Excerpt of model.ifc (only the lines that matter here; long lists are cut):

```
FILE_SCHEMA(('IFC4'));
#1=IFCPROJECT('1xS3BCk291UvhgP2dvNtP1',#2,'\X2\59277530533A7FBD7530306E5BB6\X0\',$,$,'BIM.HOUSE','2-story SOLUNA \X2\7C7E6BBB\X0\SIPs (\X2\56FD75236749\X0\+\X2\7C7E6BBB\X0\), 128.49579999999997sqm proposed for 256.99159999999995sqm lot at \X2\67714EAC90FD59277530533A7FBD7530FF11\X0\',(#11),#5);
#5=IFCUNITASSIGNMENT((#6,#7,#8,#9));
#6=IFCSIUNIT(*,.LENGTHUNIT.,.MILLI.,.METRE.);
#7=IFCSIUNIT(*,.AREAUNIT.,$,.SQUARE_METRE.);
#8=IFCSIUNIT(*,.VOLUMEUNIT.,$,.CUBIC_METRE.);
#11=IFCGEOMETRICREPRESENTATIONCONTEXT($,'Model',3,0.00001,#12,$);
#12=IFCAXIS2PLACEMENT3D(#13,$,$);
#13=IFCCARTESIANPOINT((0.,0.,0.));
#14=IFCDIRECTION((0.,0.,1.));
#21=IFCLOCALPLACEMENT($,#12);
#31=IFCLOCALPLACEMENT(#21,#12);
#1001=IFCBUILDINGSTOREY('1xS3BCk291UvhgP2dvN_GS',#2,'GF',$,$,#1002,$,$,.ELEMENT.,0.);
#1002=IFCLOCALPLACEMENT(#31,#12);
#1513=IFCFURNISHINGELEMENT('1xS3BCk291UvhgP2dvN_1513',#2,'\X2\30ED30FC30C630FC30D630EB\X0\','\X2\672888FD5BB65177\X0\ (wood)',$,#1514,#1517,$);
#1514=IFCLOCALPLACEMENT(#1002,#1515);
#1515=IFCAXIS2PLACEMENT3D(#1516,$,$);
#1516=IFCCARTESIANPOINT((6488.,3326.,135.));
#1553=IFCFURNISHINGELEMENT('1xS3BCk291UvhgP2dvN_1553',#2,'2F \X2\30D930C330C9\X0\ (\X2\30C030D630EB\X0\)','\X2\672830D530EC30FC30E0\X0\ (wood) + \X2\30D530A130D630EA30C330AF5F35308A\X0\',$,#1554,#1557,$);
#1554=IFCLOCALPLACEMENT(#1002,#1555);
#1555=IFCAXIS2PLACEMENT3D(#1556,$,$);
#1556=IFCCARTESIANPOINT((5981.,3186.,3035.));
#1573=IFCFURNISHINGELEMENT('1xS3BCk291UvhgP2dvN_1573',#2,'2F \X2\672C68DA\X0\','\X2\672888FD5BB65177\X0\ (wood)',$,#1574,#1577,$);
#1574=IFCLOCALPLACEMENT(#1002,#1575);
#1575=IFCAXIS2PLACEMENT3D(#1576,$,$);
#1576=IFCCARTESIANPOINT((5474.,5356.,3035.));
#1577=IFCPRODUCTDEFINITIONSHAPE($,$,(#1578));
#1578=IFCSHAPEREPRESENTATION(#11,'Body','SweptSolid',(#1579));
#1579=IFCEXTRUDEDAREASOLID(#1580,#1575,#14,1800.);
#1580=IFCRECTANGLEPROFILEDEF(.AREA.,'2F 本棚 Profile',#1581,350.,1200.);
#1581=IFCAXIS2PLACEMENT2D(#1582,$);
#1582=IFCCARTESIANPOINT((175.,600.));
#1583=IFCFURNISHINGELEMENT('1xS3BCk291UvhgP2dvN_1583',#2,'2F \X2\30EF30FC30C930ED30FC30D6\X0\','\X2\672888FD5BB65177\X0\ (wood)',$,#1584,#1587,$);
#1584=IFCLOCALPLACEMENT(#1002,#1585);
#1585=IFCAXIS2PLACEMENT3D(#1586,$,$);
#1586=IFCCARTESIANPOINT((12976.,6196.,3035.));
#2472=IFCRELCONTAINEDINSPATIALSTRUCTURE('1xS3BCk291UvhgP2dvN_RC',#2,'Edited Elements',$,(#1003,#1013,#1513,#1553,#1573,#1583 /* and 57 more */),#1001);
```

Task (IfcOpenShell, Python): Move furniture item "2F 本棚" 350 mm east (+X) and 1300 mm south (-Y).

```python
import ifcopenshell
import ifcopenshell.api.geometry
import ifcopenshell.util.placement

model = ifcopenshell.open("model.ifc")

item = model.by_guid("1xS3BCk291UvhgP2dvN_1573")
matrix = ifcopenshell.util.placement.get_local_placement(item.ObjectPlacement)
matrix[0, 3] += 350.0
matrix[1, 3] -= 1300.0
ifcopenshell.api.geometry.edit_object_placement(model, product=item, matrix=matrix, is_si=False)

print(ifcopenshell.util.placement.get_local_placement(item.ObjectPlacement).round(3) + 0.0)

model.write("model_updated.ifc")
```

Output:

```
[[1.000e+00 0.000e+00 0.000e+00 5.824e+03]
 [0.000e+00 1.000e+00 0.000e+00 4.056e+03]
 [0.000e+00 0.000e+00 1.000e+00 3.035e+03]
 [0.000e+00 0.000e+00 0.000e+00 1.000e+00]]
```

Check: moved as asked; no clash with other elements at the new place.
